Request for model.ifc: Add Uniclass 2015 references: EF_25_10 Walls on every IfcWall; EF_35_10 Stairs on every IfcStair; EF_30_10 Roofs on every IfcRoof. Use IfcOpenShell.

First a look at what the model holds.

```python
import ifcopenshell

model = ifcopenshell.open("model.ifc")
print(model.schema)
print("classifications:", [c.Name for c in model.by_type("IfcClassification")])
for ifc_class in ("IfcDoor", "IfcRoof", "IfcStair", "IfcWall", "IfcWindow"):
    print(ifc_class, len(model.by_type(ifc_class)))
```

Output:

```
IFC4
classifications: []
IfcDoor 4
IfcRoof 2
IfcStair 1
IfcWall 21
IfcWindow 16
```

```python
import ifcopenshell
import ifcopenshell.api.classification

model = ifcopenshell.open("model.ifc")

system = ifcopenshell.api.classification.add_classification(model, classification="Uniclass 2015")

codes = {
    "IfcWall": ("EF_25_10", "Walls"),
    "IfcStair": ("EF_35_10", "Stairs"),
    "IfcRoof": ("EF_30_10", "Roofs"),
}
for ifc_class, (code, name) in codes.items():
    products = model.by_type(ifc_class)
    ifcopenshell.api.classification.add_reference(
        model, products=products, classification=system, identification=code, name=name
    )
    print(code, len(products))

model.write("model_updated.ifc")
```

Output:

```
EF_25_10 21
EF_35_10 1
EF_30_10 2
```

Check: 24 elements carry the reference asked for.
